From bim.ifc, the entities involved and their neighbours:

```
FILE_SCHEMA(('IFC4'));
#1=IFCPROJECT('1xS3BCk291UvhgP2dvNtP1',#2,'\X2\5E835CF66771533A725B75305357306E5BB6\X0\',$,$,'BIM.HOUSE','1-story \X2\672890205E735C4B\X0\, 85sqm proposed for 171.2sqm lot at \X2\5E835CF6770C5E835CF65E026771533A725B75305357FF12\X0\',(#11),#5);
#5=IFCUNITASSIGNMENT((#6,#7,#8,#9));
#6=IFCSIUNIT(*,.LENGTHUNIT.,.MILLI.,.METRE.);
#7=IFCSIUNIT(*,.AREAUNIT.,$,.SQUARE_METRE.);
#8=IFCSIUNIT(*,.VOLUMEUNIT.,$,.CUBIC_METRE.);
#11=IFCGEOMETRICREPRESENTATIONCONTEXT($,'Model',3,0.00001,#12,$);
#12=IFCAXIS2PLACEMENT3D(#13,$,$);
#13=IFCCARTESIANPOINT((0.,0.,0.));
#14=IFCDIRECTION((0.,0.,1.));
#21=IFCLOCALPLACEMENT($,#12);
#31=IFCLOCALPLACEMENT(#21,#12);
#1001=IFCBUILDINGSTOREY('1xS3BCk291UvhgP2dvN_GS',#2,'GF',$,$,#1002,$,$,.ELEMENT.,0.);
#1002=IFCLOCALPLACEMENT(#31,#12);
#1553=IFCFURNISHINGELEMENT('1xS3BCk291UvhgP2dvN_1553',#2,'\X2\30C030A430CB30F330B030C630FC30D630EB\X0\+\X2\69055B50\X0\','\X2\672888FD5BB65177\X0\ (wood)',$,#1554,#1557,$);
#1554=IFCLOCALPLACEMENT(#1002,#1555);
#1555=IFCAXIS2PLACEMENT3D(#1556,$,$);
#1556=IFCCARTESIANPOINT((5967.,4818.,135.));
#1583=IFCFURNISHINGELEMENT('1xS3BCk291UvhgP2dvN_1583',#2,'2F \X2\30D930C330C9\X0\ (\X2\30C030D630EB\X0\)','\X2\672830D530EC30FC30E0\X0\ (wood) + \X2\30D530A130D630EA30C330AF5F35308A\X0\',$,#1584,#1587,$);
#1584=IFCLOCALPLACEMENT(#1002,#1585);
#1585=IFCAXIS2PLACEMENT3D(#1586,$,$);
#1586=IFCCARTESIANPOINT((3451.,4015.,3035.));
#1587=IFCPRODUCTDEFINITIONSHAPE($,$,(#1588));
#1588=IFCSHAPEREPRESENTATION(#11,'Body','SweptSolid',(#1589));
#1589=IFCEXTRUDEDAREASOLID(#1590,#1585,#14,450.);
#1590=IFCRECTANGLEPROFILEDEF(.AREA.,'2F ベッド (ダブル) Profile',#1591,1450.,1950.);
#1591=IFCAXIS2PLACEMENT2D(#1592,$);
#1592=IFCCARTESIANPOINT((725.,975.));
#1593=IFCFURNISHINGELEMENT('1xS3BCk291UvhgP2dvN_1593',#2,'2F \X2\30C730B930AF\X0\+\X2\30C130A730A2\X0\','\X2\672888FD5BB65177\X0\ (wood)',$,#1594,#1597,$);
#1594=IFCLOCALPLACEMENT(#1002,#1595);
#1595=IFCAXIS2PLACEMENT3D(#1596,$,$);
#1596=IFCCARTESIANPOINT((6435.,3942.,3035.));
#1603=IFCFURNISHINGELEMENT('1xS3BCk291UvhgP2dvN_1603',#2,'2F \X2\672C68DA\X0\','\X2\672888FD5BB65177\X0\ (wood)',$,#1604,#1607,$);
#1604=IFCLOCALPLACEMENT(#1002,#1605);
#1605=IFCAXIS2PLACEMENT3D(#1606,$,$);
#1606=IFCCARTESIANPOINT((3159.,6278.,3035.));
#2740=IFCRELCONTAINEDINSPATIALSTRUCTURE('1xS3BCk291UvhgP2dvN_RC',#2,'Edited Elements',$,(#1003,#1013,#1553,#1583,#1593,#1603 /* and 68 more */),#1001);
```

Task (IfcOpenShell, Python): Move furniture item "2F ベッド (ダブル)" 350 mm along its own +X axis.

```python
import ifcopenshell
import ifcopenshell.api.geometry
import ifcopenshell.util.placement
import ifcopenshell.util.unit

model = ifcopenshell.open("bim.ifc")
unit_scale = ifcopenshell.util.unit.calculate_unit_scale(model)

item = model.by_guid("1xS3BCk291UvhgP2dvN_1583")
matrix = ifcopenshell.util.placement.get_local_placement(item.ObjectPlacement)
matrix[:3, 3] += matrix[:3, 0] * 0.35 / unit_scale
ifcopenshell.api.geometry.edit_object_placement(model, product=item, matrix=matrix, is_si=False)

print(ifcopenshell.util.placement.get_local_placement(item.ObjectPlacement).round(3) + 0.0)

model.write("bim_v2.ifc")
```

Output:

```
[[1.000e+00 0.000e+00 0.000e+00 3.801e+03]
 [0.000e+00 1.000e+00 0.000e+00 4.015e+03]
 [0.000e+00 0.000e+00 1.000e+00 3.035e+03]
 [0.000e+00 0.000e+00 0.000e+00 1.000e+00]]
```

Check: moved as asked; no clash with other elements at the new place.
